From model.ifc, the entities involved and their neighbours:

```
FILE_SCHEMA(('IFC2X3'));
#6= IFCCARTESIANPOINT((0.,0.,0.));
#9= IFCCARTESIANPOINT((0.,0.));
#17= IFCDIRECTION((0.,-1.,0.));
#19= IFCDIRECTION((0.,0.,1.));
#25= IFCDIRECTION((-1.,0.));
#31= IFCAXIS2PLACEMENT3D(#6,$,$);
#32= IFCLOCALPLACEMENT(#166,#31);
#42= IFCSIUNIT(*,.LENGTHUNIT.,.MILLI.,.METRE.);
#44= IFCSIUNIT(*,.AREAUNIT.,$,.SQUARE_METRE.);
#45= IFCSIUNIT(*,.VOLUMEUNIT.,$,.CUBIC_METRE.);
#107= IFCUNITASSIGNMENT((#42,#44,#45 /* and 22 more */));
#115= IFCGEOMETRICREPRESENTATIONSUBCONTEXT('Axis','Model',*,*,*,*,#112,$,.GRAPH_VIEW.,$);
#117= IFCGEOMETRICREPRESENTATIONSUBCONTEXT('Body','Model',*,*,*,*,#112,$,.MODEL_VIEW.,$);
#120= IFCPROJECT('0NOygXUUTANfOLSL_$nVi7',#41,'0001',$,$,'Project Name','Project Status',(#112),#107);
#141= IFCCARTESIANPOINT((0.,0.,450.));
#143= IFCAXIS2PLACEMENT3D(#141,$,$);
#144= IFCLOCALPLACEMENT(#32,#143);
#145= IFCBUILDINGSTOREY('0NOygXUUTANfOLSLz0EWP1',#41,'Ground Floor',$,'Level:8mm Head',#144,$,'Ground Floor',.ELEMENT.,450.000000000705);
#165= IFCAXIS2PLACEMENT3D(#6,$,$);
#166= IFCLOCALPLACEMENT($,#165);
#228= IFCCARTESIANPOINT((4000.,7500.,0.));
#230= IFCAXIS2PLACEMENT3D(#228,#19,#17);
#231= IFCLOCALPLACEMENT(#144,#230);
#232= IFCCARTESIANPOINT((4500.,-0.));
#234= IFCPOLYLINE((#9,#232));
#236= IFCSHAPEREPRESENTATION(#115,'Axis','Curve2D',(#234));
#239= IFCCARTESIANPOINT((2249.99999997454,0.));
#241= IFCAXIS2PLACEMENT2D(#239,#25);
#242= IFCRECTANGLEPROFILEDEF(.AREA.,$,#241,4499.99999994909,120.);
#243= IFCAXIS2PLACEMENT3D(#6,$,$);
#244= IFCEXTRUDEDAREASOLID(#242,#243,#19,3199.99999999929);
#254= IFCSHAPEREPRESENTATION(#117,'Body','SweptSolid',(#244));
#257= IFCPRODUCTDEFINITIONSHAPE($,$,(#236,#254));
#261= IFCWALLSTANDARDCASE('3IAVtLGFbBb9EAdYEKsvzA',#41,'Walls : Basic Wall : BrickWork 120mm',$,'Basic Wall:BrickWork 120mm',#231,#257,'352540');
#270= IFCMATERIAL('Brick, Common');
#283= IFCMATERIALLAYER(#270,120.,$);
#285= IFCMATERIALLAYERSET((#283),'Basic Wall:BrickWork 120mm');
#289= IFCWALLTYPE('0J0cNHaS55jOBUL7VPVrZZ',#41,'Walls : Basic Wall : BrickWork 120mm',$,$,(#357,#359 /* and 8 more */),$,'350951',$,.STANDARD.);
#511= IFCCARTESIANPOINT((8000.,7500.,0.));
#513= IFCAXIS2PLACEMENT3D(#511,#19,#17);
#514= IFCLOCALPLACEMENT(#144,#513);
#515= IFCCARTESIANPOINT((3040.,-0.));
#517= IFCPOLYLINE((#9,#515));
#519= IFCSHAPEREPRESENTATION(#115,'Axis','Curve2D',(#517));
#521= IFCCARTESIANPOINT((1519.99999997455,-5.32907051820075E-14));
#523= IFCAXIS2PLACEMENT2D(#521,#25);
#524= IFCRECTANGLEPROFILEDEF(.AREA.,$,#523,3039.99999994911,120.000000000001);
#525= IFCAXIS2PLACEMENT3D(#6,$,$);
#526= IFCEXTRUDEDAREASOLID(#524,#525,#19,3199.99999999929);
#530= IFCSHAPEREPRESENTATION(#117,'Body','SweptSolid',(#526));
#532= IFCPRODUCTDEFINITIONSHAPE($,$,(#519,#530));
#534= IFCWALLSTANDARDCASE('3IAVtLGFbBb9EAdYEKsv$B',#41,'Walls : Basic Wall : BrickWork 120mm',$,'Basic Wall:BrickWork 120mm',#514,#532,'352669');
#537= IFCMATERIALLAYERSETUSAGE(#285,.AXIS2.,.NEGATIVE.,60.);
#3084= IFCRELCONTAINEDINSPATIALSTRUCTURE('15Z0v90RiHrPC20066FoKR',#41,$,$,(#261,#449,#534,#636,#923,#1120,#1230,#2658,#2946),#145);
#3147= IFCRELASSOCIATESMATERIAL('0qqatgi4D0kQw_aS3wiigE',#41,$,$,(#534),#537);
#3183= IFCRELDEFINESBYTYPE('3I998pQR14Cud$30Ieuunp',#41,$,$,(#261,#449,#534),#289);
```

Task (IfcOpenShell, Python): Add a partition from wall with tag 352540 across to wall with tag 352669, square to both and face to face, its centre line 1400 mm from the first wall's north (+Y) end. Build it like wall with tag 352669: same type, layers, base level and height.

```python
import numpy as np
import ifcopenshell
import ifcopenshell.api.geometry
import ifcopenshell.api.material
import ifcopenshell.api.pset
import ifcopenshell.api.root
import ifcopenshell.api.spatial
import ifcopenshell.api.type
import ifcopenshell.geom
import ifcopenshell.util.element
import ifcopenshell.util.placement
import ifcopenshell.util.representation
import ifcopenshell.util.shape
import ifcopenshell.util.unit

model = ifcopenshell.open("model.ifc")
unit_scale = ifcopenshell.util.unit.calculate_unit_scale(model)
settings = ifcopenshell.geom.settings()
settings.set("use-world-coords", True)

start_wall = model.by_guid("3IAVtLGFbBb9EAdYEKsvzA")
end_wall = model.by_id(534)
like = model.by_guid("3IAVtLGFbBb9EAdYEKsv$B")
matrix = ifcopenshell.util.placement.get_local_placement(start_wall.ObjectPlacement)
matrix[:3, 3] *= unit_scale


def extent(element):
    """Bounding box in the first wall's axes, in metres."""
    shape = ifcopenshell.geom.create_shape(settings, element)
    points = (ifcopenshell.util.shape.get_vertices(shape.geometry) - matrix[:3, 3]) @ matrix[:3, :3]
    return points.min(axis=0), points.max(axis=0)


y_start = extent(start_wall)[1][1]
y_end = extent(end_wall)[0][1]
like_min, like_max = extent(like)
length, height = float(abs(y_end - y_start)), float(like_max[2] - like_min[2])
layer_set = ifcopenshell.util.element.get_material(like, should_skip_usage=True)
thickness = sum(layer.LayerThickness for layer in layer_set.MaterialLayers) * unit_scale

wall = ifcopenshell.api.root.create_entity(model, ifc_class="IfcWallStandardCase", name="New partition")
storey = ifcopenshell.util.element.get_container(like)
ifcopenshell.api.spatial.assign_container(model, products=[wall], relating_structure=storey)
ifcopenshell.api.type.assign_type(
    model, related_objects=[wall], relating_type=ifcopenshell.util.element.get_type(like), should_map_representations=False
)
rel = ifcopenshell.api.material.assign_material(
    model, products=[wall], type="IfcMaterialLayerSetUsage", material=layer_set
)
rel.RelatingMaterial.OffsetFromReferenceLine = -thickness / 2 / unit_scale
pset = ifcopenshell.api.pset.add_pset(model, product=wall, name="Pset_WallCommon")
ifcopenshell.api.pset.edit_pset(model, pset=pset, properties={"IsExternal": False, "LoadBearing": False})

# The axis runs down the middle of the wall.
axis = ifcopenshell.api.geometry.add_axis_representation(
    model, context=ifcopenshell.util.representation.get_context(model, "Model", "Axis"), axis=[(0.0, 0.0), (length, 0.0)]
)
body = ifcopenshell.api.geometry.add_wall_representation(
    model,
    context=ifcopenshell.util.representation.get_context(model, "Model", "Body", "MODEL_VIEW"),
    length=length,
    height=height,
    thickness=thickness,
    offset=-thickness / 2,
)
for representation in (axis, body):
    ifcopenshell.api.geometry.assign_representation(model, product=wall, representation=representation)

placement = matrix @ ifcopenshell.util.placement.rotation(90, "Z")
placement[:, 3] = matrix @ np.array([extent(start_wall)[0][0] + 1.4, y_start, like_min[2], 1.0])
ifcopenshell.api.geometry.edit_object_placement(model, product=wall, matrix=placement)

print(f"partition {length:.3f} m long, {height:.3f} m high, {thickness:.3f} m thick")

model.write("model_edited.ifc")
```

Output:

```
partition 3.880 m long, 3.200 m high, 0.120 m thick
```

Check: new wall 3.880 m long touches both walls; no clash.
